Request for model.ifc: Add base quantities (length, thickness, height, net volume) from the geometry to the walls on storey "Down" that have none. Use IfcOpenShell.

First a look at what the model holds.

```python
import ifcopenshell
import ifcopenshell.util.element
import ifcopenshell.util.unit

model = ifcopenshell.open("model.ifc")
print(model.schema)
for unit_type in ("LENGTHUNIT", "AREAUNIT", "VOLUMEUNIT"):
    print(unit_type, ifcopenshell.util.unit.calculate_unit_scale(model, unit_type))
storey = next(s for s in model.by_type("IfcBuildingStorey") if s.Name == "Down")
walls = [e for e in ifcopenshell.util.element.get_decomposition(storey) if e.is_a("IfcWall")]
for e in sorted(walls, key=lambda e: e.id()):
    print(e.id(), e.is_a(), e.Name, list(ifcopenshell.util.element.get_psets(e, qtos_only=True)), sep=" | ")
```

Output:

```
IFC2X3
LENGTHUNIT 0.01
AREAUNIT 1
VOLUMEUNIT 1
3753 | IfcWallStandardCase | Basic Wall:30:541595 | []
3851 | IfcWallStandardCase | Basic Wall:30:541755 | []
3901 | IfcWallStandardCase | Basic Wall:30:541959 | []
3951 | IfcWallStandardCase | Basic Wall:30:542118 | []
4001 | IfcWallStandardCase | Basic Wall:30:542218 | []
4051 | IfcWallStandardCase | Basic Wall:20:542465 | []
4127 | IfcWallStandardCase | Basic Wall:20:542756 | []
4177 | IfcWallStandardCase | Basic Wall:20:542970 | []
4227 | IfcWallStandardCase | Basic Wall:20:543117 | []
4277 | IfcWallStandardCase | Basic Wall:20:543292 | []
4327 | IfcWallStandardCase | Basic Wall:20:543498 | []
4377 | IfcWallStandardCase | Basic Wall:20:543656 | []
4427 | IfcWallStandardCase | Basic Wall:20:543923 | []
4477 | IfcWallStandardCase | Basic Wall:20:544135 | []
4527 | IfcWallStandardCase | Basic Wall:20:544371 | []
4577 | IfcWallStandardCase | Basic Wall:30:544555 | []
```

```python
import ifcopenshell
import ifcopenshell.api.pset
import ifcopenshell.geom
import ifcopenshell.util.element
import ifcopenshell.util.shape
import ifcopenshell.util.unit

model = ifcopenshell.open("model.ifc")
unit_scale = ifcopenshell.util.unit.calculate_unit_scale(model)
volume_scale = ifcopenshell.util.unit.calculate_unit_scale(model, "VOLUMEUNIT")
settings = ifcopenshell.geom.settings()

storey = next(s for s in model.by_type("IfcBuildingStorey") if s.Name == "Down")
walls = [e for e in ifcopenshell.util.element.get_decomposition(storey) if e.is_a("IfcWall")]

for e in sorted(walls, key=lambda e: e.id()):
    if ifcopenshell.util.element.get_psets(e, qtos_only=True, should_inherit=False):
        continue
    # Geometry comes back in metres, in the element's own axes.
    shape = ifcopenshell.geom.create_shape(settings, e)
    values = {
        "Length": ifcopenshell.util.shape.get_x(shape.geometry) / unit_scale,
        "Width": ifcopenshell.util.shape.get_y(shape.geometry) / unit_scale,
        "Height": ifcopenshell.util.shape.get_z(shape.geometry) / unit_scale,
        "NetVolume": ifcopenshell.util.shape.get_volume(shape.geometry) / volume_scale,
    }
    qto = ifcopenshell.api.pset.add_qto(model, product=e, name="BaseQuantities")
    ifcopenshell.api.pset.edit_qto(model, qto=qto, properties=values)
    print(e.id(), {k: round(v, 3) for k, v in values.items()})

model.write("model_updated.ifc")
```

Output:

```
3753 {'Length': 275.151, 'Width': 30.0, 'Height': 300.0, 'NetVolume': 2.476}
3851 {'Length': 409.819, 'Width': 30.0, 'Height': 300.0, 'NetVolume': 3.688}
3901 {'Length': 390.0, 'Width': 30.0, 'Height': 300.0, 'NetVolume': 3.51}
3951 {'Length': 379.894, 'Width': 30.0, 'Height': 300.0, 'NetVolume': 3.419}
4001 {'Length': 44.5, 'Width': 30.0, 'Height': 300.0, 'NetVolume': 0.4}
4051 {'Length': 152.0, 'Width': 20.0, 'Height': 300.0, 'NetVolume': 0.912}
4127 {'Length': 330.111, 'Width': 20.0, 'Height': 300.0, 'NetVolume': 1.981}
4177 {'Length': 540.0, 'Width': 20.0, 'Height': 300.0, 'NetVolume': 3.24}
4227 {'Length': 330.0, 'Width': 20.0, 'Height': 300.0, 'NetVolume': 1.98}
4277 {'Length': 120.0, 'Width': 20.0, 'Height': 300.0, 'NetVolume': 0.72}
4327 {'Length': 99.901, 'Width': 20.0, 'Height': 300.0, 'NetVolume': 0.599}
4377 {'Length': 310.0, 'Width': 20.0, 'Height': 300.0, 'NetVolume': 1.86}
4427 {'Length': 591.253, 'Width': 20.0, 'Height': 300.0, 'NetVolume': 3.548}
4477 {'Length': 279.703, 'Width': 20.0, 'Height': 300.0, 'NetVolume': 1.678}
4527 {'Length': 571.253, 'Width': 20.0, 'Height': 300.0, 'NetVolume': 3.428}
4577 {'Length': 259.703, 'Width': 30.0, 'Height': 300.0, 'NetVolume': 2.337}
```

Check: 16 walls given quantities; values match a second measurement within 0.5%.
